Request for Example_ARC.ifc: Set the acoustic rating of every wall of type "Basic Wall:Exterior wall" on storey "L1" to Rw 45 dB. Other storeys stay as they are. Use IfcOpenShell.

First a look at what the model holds.

```python
import ifcopenshell
import ifcopenshell.util.element

model = ifcopenshell.open("Example_ARC.ifc")
print(model.schema)
storey = next(s for s in model.by_type("IfcBuildingStorey") if s.Name == "L1")
walls = [e for e in ifcopenshell.util.element.get_decomposition(storey) if e.is_a("IfcWall")]
seen = {}
for e in walls:
    element_type = ifcopenshell.util.element.get_type(e)
    key = (element_type.Name if element_type != e and element_type else None, ifcopenshell.util.element.get_pset(e, "Pset_WallCommon", "AcousticRating"))
    seen[key] = seen.get(key, 0) + 1
for (name, value), count in sorted(seen.items(), key=str):
    print(count, "x", name, "|", value)
```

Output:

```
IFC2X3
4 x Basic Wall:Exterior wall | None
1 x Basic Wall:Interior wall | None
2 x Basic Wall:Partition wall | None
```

```python
import ifcopenshell
import ifcopenshell.api.pset
import ifcopenshell.util.element

model = ifcopenshell.open("Example_ARC.ifc")

storey = next(s for s in model.by_type("IfcBuildingStorey") if s.Name == "L1")
walls = [e for e in ifcopenshell.util.element.get_decomposition(storey) if e.is_a("IfcWall")]

count = 0
for e in walls:
    element_type = ifcopenshell.util.element.get_type(e)
    if element_type in (None, e) or element_type.Name != "Basic Wall:Exterior wall":
        continue
    # add_pset returns the element's existing set when there is one.
    pset = ifcopenshell.api.pset.add_pset(model, product=e, name="Pset_WallCommon")
    ifcopenshell.api.pset.edit_pset(model, pset=pset, properties={"AcousticRating": "Rw 45 dB"})
    count += 1

print(count, "walls updated")

model.write("Example_ARC_edited.ifc")
```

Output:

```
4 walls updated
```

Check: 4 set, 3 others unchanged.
